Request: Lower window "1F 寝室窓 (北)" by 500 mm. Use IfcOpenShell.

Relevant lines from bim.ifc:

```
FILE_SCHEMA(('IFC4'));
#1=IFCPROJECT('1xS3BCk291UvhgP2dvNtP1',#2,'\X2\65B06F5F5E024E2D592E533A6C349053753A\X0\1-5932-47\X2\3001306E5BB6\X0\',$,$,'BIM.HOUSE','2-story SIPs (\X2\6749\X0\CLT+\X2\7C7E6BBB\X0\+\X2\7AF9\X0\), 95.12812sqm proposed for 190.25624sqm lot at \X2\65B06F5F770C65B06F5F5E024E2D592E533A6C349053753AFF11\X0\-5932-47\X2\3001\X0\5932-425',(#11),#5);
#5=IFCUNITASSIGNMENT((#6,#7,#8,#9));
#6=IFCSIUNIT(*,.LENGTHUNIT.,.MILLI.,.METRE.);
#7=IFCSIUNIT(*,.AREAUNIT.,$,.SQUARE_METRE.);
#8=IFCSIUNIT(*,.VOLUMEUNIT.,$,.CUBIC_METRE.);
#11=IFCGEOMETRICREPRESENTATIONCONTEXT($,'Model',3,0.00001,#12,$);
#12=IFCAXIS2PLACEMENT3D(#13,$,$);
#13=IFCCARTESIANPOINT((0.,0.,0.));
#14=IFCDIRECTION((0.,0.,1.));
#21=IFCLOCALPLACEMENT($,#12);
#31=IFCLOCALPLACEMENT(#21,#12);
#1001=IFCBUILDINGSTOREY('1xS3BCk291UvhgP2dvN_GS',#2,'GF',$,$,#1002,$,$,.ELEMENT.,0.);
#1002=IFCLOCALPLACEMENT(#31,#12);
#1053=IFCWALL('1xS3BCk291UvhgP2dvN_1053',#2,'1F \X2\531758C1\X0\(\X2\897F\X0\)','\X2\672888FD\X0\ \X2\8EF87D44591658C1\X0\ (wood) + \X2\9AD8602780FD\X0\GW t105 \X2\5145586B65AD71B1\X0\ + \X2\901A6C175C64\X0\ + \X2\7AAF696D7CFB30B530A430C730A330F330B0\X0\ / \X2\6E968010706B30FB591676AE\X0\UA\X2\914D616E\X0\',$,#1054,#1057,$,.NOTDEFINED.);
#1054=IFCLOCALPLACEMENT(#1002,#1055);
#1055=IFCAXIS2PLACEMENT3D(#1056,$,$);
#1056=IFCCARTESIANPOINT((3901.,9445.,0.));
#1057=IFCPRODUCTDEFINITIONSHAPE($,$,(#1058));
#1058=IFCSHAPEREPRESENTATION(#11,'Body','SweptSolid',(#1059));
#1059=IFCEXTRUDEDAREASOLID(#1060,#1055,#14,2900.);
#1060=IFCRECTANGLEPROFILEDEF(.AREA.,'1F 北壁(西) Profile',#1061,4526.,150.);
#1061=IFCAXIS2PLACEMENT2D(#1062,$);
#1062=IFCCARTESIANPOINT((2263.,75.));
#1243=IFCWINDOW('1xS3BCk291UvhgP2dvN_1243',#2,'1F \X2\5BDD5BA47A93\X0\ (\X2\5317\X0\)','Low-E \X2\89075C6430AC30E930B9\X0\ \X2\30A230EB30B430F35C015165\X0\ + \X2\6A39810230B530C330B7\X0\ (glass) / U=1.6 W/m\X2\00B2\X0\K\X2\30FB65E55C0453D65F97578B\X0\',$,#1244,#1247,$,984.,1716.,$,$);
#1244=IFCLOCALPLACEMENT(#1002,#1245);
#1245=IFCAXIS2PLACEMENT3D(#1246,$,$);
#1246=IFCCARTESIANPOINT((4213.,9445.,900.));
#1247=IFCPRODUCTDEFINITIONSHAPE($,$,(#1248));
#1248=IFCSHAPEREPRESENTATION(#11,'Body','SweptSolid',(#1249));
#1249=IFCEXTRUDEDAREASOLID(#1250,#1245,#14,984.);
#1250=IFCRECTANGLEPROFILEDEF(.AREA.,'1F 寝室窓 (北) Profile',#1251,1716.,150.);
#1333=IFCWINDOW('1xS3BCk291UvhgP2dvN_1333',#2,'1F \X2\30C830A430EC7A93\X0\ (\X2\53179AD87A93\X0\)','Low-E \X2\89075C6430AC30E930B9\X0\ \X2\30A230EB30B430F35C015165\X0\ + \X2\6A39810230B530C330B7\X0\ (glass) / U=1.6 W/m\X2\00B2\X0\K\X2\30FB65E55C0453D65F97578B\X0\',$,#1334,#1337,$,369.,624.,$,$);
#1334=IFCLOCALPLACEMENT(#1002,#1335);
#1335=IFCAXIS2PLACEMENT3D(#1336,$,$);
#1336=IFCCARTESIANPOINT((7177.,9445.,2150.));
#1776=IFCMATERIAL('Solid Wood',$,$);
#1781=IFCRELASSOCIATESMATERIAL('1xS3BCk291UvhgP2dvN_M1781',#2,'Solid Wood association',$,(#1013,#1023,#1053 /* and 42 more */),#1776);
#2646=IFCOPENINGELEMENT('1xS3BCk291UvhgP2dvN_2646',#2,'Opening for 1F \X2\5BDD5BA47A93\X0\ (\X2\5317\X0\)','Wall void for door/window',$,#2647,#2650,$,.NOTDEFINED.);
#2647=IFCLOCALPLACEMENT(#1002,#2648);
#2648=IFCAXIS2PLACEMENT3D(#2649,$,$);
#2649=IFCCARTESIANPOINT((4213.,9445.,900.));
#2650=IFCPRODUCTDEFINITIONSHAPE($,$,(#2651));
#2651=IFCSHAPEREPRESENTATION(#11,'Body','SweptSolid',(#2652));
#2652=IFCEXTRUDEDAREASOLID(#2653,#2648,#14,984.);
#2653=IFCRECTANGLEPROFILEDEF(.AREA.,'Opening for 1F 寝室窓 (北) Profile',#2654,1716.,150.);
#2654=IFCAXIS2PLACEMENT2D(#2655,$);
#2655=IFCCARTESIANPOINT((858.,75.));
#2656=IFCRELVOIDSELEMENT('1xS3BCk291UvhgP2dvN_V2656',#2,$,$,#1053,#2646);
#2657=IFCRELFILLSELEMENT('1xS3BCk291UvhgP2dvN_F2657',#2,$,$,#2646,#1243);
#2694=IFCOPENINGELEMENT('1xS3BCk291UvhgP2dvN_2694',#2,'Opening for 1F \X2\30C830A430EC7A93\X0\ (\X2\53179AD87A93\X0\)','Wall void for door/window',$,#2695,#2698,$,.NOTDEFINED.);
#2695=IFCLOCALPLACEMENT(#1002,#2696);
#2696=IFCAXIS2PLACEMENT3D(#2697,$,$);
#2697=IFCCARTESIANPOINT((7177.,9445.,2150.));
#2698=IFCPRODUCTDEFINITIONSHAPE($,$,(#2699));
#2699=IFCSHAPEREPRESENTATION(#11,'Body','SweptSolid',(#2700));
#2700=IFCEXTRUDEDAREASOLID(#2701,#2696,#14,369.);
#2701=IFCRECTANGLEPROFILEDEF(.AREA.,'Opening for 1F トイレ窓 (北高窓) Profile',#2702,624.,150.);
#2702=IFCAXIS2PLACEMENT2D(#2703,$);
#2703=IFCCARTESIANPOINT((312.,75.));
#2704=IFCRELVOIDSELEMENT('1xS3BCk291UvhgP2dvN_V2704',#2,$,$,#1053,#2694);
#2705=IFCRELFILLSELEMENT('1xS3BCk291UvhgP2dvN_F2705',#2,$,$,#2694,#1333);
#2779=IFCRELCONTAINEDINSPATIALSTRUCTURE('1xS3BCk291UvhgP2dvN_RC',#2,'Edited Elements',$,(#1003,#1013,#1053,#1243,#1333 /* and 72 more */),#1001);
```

```python
import numpy as np
import ifcopenshell
import ifcopenshell.api.geometry
import ifcopenshell.util.placement
import ifcopenshell.util.unit

model = ifcopenshell.open("bim.ifc")
unit_scale = ifcopenshell.util.unit.calculate_unit_scale(model)

window = model.by_guid("1xS3BCk291UvhgP2dvN_1243")
opening = window.FillsVoids[0].RelatingOpeningElement
dz = -0.5 / unit_scale

shift = np.array([0.0, 0.0, dz])
# The window is not placed relative to its opening, so move both.
for product in (opening, window):
    matrix = ifcopenshell.util.placement.get_local_placement(product.ObjectPlacement)
    matrix[:3, 3] += shift
    ifcopenshell.api.geometry.edit_object_placement(model, product=product, matrix=matrix, is_si=False)

print(f"moved by {dz * unit_scale:+.3f} m")

model.write("bim_v2.ifc")
```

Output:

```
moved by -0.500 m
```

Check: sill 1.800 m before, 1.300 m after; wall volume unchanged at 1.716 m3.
